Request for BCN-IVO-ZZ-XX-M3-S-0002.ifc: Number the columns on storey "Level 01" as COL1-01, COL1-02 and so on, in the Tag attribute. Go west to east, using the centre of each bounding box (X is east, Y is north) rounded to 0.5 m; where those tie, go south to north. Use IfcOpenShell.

First a look at what the model holds.

```python
import ifcopenshell
import ifcopenshell.util.element
import ifcopenshell.util.placement

model = ifcopenshell.open("BCN-IVO-ZZ-XX-M3-S-0002.ifc")
print(model.schema)
storey = next(s for s in model.by_type("IfcBuildingStorey") if s.Name == "Level 01")
columns = [e for e in ifcopenshell.util.element.get_decomposition(storey) if e.is_a("IfcColumn")]
for e in sorted(columns, key=lambda e: e.id()):
    origin = ifcopenshell.util.placement.get_local_placement(e.ObjectPlacement)[:3, 3]
    print(e.id(), e.Tag, e.Name, origin.round(2) + 0.0, sep=" | ")
```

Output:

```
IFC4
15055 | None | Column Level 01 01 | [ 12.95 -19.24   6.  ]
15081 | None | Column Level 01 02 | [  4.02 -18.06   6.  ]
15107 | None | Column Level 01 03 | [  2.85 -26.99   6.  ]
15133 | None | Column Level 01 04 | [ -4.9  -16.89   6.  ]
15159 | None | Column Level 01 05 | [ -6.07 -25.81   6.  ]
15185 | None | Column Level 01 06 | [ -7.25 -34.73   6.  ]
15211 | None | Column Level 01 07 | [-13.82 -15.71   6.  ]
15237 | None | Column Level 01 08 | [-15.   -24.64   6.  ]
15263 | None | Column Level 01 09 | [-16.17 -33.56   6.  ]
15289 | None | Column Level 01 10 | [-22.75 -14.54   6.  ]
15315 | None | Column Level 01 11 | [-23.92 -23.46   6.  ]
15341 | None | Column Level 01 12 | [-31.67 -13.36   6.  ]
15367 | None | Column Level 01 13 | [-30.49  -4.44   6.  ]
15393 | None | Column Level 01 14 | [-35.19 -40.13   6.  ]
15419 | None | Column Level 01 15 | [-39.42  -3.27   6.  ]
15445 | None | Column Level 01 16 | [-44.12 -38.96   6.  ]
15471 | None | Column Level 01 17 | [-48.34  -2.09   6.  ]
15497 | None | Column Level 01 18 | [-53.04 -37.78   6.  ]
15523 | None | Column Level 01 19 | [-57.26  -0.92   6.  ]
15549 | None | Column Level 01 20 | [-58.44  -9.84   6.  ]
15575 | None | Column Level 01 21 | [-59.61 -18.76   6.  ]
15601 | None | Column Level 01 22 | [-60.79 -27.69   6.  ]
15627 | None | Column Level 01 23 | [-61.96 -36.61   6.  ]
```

```python
import ifcopenshell
import ifcopenshell.geom
import ifcopenshell.util.element
import ifcopenshell.util.shape

model = ifcopenshell.open("BCN-IVO-ZZ-XX-M3-S-0002.ifc")
settings = ifcopenshell.geom.settings()
settings.set("use-world-coords", True)


def centre(element):
    shape = ifcopenshell.geom.create_shape(settings, element)
    return ifcopenshell.util.shape.get_bbox_centroid(shape.geometry)


storey = next(s for s in model.by_type("IfcBuildingStorey") if s.Name == "Level 01")
columns = [e for e in ifcopenshell.util.element.get_decomposition(storey) if e.is_a("IfcColumn")]

# Insertion points can sit at a corner or the storey origin, so sort by the geometry (in metres).
centres = {e: centre(e) for e in columns}
columns.sort(key=lambda e: (round(centres[e][0] / 0.5), centres[e][1]))

for i, e in enumerate(columns, start=1):
    number = f"COL1-{i:02d}"
    e.Tag = number
    print(e.id(), number)

model.write("BCN-IVO-ZZ-XX-M3-S-0002-out.ifc")
```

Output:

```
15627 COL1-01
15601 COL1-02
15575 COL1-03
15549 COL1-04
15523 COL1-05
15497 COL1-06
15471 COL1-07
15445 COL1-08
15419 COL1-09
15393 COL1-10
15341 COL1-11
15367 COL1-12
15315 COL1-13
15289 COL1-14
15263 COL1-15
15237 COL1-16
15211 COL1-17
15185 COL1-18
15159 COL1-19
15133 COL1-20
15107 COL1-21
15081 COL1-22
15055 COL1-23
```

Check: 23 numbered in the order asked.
